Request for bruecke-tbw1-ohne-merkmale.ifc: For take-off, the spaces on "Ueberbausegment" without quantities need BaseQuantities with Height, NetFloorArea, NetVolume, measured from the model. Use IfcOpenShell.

First a look at what the model holds.

```python
import ifcopenshell
import ifcopenshell.util.element
import ifcopenshell.util.unit

model = ifcopenshell.open("bruecke-tbw1-ohne-merkmale.ifc")
print(model.schema)
for unit_type in ("LENGTHUNIT", "AREAUNIT", "VOLUMEUNIT"):
    print(unit_type, ifcopenshell.util.unit.calculate_unit_scale(model, unit_type))
storey = next(s for s in model.by_type("IfcBuildingStorey") if s.Name == "Ueberbausegment")
spaces = [e for e in ifcopenshell.util.element.get_decomposition(storey) if e.is_a("IfcSpace")]
for e in sorted(spaces, key=lambda e: e.id()):
    print(e.id(), e.is_a(), e.Name, list(ifcopenshell.util.element.get_psets(e, qtos_only=True)), sep=" | ")
```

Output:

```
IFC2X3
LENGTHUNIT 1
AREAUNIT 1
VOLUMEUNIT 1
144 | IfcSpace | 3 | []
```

```python
import ifcopenshell
import ifcopenshell.api.pset
import ifcopenshell.geom
import ifcopenshell.util.element
import ifcopenshell.util.shape
import ifcopenshell.util.unit

model = ifcopenshell.open("bruecke-tbw1-ohne-merkmale.ifc")
unit_scale = ifcopenshell.util.unit.calculate_unit_scale(model)
area_scale = ifcopenshell.util.unit.calculate_unit_scale(model, "AREAUNIT")
volume_scale = ifcopenshell.util.unit.calculate_unit_scale(model, "VOLUMEUNIT")
settings = ifcopenshell.geom.settings()

storey = next(s for s in model.by_type("IfcBuildingStorey") if s.Name == "Ueberbausegment")
spaces = [e for e in ifcopenshell.util.element.get_decomposition(storey) if e.is_a("IfcSpace")]

for e in sorted(spaces, key=lambda e: e.id()):
    if ifcopenshell.util.element.get_psets(e, qtos_only=True, should_inherit=False):
        continue
    # Geometry comes back in metres, in the element's own axes.
    shape = ifcopenshell.geom.create_shape(settings, e)
    values = {
        "Height": ifcopenshell.util.shape.get_z(shape.geometry) / unit_scale,
        "NetFloorArea": ifcopenshell.util.shape.get_footprint_area(shape.geometry) / area_scale,
        "NetVolume": ifcopenshell.util.shape.get_volume(shape.geometry) / volume_scale,
    }
    qto = ifcopenshell.api.pset.add_qto(model, product=e, name="BaseQuantities")
    ifcopenshell.api.pset.edit_qto(model, qto=qto, properties=values)
    print(e.id(), {k: round(v, 3) for k, v in values.items()})

model.write("bruecke-tbw1-ohne-merkmale_rev.ifc")
```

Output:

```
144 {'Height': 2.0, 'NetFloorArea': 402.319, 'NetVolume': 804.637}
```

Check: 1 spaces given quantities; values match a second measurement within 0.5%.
